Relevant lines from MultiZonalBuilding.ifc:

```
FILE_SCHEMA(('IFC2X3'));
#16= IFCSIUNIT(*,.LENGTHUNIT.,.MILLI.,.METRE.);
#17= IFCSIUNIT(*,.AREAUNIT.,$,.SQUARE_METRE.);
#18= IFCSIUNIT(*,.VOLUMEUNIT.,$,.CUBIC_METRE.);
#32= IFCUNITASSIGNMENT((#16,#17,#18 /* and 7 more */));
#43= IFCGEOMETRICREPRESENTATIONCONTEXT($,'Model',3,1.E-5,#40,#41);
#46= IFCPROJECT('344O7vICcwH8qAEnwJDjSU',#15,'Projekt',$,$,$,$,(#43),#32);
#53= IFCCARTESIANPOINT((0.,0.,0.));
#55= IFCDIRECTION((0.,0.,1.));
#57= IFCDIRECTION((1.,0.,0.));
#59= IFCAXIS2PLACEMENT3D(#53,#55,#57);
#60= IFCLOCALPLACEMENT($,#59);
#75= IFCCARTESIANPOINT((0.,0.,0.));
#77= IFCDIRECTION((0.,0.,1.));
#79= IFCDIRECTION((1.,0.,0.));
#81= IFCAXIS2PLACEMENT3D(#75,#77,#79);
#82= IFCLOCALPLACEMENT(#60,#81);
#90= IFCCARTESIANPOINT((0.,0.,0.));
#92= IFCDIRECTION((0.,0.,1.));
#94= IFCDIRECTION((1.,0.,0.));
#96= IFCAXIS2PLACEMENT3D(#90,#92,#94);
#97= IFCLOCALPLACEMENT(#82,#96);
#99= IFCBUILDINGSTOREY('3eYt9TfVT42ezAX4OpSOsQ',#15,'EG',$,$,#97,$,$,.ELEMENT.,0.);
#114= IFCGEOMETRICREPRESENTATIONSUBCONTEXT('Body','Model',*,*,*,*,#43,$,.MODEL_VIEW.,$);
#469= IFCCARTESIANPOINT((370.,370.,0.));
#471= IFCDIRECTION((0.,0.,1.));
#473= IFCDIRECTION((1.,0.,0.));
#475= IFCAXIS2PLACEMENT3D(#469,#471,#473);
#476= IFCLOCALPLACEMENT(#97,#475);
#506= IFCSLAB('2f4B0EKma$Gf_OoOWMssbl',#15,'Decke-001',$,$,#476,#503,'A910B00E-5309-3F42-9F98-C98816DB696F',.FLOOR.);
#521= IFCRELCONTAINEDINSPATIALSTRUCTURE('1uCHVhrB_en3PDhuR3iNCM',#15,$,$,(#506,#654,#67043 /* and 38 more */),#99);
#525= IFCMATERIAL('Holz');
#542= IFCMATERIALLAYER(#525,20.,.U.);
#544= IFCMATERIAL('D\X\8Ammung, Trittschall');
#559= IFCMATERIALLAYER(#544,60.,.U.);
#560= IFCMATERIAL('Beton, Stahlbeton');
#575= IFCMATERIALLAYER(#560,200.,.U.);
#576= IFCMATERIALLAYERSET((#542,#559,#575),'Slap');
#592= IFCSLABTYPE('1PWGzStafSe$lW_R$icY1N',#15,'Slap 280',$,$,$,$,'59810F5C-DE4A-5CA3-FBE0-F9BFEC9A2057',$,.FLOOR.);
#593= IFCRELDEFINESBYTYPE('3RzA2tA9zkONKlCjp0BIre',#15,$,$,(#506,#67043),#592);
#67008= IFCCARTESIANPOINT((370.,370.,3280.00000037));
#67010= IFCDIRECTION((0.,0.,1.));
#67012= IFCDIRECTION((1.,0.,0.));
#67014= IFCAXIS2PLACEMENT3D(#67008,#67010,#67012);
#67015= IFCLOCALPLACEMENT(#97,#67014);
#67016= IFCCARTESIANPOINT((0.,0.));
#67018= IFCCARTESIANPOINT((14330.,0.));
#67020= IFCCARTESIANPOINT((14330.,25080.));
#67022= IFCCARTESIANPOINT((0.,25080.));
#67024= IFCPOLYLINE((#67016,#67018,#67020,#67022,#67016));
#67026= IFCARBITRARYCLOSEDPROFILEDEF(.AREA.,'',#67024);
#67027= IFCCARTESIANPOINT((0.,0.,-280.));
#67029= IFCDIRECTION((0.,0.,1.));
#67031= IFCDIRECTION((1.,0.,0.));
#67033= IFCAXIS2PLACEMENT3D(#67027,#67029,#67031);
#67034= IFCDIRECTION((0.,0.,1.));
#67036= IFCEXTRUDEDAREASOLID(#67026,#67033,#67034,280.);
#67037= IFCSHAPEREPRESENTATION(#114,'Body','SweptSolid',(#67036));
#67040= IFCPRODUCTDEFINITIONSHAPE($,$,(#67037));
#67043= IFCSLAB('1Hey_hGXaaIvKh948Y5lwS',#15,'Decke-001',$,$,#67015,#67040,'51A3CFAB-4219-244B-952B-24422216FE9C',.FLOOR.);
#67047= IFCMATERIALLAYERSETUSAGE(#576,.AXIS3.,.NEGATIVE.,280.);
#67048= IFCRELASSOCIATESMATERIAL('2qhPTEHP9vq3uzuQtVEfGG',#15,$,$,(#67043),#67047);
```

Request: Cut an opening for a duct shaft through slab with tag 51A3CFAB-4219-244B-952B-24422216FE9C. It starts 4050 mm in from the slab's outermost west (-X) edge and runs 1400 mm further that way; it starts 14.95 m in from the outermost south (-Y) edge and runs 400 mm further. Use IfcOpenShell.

```python
import numpy as np
import ifcopenshell
import ifcopenshell.api.feature
import ifcopenshell.api.geometry
import ifcopenshell.api.root
import ifcopenshell.geom
import ifcopenshell.util.placement
import ifcopenshell.util.representation
import ifcopenshell.util.shape
import ifcopenshell.util.unit

model = ifcopenshell.open("MultiZonalBuilding.ifc")
unit_scale = ifcopenshell.util.unit.calculate_unit_scale(model)
settings = ifcopenshell.geom.settings()


def volume(element):
    """Net volume in cubic metres, openings subtracted."""
    shape = ifcopenshell.geom.create_shape(settings, element)
    return ifcopenshell.util.shape.get_volume(shape.geometry)


slab = model.by_id(67043)
before = volume(slab)

# Extent in the slab's own axes, in metres. The edges named are its -X and -Y sides.
slab_shape = ifcopenshell.geom.create_shape(settings, slab)
vertices = ifcopenshell.util.shape.get_vertices(slab_shape.geometry)
x_min, y_min, bottom = vertices.min(axis=0)
top = vertices[:, 2].max()

opening = ifcopenshell.api.root.create_entity(model, ifc_class="IfcOpeningElement", name="Duct shaft opening")
context = ifcopenshell.util.representation.get_context(model, "Model", "Body", "MODEL_VIEW")
width, depth = 1.4, 0.4
outline = [(0.0, 0.0), (width, 0.0), (width, depth), (0.0, depth), (0.0, 0.0)]
# Overshoot both faces by 50 mm so the cut is clean.
shape = ifcopenshell.api.geometry.add_slab_representation(
    model, context=context, depth=top - bottom + 0.1, polyline=outline
)
ifcopenshell.api.geometry.assign_representation(model, product=opening, representation=shape)

matrix = ifcopenshell.util.placement.get_local_placement(slab.ObjectPlacement)
matrix[:, 3] = matrix @ np.append(np.array([x_min + 4.05, y_min + 14.95, bottom - 0.05]) / unit_scale, 1.0)
ifcopenshell.api.geometry.edit_object_placement(model, product=opening, matrix=matrix, is_si=False)
ifcopenshell.api.feature.add_feature(model, feature=opening, element=slab)

after = volume(slab)

print(f"slab volume {before:.3f} -> {after:.3f} m3")

model.write("MultiZonalBuilding_rev.ifc")
```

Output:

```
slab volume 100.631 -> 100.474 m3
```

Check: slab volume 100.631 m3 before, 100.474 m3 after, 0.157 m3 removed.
